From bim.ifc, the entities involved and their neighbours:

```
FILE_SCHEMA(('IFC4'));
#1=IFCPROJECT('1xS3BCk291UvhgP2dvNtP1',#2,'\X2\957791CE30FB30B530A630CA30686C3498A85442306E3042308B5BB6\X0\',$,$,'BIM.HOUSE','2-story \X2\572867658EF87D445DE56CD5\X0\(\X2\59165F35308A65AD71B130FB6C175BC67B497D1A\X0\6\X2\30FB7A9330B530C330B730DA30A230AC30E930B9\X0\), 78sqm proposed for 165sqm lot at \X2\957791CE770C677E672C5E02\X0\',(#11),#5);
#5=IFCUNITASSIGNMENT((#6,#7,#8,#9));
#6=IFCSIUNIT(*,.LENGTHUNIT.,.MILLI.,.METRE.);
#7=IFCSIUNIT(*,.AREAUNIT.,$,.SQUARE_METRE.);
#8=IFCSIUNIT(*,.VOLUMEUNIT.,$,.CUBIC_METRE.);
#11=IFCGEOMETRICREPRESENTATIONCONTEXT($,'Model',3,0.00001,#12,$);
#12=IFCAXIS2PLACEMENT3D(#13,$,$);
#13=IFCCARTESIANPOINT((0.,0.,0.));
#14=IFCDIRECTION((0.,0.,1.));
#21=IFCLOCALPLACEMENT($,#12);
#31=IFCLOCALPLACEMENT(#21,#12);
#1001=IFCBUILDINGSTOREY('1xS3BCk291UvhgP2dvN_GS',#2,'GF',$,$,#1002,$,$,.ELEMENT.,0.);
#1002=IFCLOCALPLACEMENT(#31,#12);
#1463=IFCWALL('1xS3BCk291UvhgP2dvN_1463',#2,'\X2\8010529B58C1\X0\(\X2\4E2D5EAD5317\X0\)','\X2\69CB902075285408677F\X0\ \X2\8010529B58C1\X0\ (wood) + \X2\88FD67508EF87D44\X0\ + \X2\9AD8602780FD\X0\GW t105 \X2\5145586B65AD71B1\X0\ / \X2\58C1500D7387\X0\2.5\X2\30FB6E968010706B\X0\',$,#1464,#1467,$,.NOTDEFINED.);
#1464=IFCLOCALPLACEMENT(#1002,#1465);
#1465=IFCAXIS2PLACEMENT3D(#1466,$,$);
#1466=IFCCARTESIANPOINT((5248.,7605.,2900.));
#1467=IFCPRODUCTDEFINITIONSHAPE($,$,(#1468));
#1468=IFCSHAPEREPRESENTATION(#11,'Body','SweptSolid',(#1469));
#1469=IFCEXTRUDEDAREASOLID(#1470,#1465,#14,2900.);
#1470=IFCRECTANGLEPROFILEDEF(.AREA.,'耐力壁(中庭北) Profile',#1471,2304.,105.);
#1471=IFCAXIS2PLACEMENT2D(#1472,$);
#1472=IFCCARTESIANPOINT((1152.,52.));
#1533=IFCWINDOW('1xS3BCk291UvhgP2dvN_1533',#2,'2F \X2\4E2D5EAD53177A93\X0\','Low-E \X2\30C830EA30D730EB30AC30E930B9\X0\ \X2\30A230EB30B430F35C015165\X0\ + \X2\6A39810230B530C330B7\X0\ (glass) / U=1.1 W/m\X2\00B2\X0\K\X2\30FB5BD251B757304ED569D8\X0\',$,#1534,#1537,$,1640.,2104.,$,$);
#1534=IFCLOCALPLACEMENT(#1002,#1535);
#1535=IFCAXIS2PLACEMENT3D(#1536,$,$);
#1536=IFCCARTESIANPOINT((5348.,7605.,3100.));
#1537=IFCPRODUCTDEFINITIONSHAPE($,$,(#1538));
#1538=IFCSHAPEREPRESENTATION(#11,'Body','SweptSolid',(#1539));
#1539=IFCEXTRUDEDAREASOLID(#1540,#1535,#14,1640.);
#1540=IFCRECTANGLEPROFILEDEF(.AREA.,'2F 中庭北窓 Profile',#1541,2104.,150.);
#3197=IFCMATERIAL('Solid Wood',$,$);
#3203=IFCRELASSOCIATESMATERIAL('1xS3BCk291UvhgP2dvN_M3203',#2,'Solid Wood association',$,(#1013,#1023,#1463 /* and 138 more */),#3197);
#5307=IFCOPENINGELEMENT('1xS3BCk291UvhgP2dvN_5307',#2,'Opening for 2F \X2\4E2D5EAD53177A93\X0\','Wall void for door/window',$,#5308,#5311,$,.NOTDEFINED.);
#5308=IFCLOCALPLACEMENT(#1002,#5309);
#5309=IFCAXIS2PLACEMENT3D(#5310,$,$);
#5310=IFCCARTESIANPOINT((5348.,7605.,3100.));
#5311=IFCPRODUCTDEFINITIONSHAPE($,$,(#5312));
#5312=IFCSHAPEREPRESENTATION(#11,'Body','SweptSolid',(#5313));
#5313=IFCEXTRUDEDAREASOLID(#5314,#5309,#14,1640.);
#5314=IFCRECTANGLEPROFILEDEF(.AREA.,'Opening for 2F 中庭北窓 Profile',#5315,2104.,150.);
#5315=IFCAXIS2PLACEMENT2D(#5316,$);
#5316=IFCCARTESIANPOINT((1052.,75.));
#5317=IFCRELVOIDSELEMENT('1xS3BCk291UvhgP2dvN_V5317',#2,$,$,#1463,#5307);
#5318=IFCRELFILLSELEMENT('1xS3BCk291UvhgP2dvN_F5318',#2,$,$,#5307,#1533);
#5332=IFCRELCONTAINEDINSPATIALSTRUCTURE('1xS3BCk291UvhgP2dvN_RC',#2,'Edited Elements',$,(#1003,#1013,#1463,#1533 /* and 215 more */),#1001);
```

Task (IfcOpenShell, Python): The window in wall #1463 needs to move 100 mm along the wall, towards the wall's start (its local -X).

```python
import ifcopenshell
import ifcopenshell.api.geometry
import ifcopenshell.util.placement
import ifcopenshell.util.unit

model = ifcopenshell.open("bim.ifc")
unit_scale = ifcopenshell.util.unit.calculate_unit_scale(model)

window = model.by_id(1533)
opening = window.FillsVoids[0].RelatingOpeningElement
wall = opening.VoidsElements[0].RelatingBuildingElement

wall_matrix = ifcopenshell.util.placement.get_local_placement(wall.ObjectPlacement)
shift = wall_matrix[:3, 0] * -0.1 / unit_scale
before = ifcopenshell.util.placement.get_local_placement(window.ObjectPlacement)[:3, 3].copy()

# The window is not placed relative to its opening, so move both.
for product in (opening, window):
    matrix = ifcopenshell.util.placement.get_local_placement(product.ObjectPlacement)
    matrix[:3, 3] += shift
    ifcopenshell.api.geometry.edit_object_placement(model, product=product, matrix=matrix, is_si=False)

after = ifcopenshell.util.placement.get_local_placement(window.ObjectPlacement)[:3, 3]
print("window moved by", (after - before).round(3) + 0.0)

model.write("bim_rev.ifc")
```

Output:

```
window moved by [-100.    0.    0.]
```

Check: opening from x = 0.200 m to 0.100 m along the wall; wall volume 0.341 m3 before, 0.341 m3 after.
